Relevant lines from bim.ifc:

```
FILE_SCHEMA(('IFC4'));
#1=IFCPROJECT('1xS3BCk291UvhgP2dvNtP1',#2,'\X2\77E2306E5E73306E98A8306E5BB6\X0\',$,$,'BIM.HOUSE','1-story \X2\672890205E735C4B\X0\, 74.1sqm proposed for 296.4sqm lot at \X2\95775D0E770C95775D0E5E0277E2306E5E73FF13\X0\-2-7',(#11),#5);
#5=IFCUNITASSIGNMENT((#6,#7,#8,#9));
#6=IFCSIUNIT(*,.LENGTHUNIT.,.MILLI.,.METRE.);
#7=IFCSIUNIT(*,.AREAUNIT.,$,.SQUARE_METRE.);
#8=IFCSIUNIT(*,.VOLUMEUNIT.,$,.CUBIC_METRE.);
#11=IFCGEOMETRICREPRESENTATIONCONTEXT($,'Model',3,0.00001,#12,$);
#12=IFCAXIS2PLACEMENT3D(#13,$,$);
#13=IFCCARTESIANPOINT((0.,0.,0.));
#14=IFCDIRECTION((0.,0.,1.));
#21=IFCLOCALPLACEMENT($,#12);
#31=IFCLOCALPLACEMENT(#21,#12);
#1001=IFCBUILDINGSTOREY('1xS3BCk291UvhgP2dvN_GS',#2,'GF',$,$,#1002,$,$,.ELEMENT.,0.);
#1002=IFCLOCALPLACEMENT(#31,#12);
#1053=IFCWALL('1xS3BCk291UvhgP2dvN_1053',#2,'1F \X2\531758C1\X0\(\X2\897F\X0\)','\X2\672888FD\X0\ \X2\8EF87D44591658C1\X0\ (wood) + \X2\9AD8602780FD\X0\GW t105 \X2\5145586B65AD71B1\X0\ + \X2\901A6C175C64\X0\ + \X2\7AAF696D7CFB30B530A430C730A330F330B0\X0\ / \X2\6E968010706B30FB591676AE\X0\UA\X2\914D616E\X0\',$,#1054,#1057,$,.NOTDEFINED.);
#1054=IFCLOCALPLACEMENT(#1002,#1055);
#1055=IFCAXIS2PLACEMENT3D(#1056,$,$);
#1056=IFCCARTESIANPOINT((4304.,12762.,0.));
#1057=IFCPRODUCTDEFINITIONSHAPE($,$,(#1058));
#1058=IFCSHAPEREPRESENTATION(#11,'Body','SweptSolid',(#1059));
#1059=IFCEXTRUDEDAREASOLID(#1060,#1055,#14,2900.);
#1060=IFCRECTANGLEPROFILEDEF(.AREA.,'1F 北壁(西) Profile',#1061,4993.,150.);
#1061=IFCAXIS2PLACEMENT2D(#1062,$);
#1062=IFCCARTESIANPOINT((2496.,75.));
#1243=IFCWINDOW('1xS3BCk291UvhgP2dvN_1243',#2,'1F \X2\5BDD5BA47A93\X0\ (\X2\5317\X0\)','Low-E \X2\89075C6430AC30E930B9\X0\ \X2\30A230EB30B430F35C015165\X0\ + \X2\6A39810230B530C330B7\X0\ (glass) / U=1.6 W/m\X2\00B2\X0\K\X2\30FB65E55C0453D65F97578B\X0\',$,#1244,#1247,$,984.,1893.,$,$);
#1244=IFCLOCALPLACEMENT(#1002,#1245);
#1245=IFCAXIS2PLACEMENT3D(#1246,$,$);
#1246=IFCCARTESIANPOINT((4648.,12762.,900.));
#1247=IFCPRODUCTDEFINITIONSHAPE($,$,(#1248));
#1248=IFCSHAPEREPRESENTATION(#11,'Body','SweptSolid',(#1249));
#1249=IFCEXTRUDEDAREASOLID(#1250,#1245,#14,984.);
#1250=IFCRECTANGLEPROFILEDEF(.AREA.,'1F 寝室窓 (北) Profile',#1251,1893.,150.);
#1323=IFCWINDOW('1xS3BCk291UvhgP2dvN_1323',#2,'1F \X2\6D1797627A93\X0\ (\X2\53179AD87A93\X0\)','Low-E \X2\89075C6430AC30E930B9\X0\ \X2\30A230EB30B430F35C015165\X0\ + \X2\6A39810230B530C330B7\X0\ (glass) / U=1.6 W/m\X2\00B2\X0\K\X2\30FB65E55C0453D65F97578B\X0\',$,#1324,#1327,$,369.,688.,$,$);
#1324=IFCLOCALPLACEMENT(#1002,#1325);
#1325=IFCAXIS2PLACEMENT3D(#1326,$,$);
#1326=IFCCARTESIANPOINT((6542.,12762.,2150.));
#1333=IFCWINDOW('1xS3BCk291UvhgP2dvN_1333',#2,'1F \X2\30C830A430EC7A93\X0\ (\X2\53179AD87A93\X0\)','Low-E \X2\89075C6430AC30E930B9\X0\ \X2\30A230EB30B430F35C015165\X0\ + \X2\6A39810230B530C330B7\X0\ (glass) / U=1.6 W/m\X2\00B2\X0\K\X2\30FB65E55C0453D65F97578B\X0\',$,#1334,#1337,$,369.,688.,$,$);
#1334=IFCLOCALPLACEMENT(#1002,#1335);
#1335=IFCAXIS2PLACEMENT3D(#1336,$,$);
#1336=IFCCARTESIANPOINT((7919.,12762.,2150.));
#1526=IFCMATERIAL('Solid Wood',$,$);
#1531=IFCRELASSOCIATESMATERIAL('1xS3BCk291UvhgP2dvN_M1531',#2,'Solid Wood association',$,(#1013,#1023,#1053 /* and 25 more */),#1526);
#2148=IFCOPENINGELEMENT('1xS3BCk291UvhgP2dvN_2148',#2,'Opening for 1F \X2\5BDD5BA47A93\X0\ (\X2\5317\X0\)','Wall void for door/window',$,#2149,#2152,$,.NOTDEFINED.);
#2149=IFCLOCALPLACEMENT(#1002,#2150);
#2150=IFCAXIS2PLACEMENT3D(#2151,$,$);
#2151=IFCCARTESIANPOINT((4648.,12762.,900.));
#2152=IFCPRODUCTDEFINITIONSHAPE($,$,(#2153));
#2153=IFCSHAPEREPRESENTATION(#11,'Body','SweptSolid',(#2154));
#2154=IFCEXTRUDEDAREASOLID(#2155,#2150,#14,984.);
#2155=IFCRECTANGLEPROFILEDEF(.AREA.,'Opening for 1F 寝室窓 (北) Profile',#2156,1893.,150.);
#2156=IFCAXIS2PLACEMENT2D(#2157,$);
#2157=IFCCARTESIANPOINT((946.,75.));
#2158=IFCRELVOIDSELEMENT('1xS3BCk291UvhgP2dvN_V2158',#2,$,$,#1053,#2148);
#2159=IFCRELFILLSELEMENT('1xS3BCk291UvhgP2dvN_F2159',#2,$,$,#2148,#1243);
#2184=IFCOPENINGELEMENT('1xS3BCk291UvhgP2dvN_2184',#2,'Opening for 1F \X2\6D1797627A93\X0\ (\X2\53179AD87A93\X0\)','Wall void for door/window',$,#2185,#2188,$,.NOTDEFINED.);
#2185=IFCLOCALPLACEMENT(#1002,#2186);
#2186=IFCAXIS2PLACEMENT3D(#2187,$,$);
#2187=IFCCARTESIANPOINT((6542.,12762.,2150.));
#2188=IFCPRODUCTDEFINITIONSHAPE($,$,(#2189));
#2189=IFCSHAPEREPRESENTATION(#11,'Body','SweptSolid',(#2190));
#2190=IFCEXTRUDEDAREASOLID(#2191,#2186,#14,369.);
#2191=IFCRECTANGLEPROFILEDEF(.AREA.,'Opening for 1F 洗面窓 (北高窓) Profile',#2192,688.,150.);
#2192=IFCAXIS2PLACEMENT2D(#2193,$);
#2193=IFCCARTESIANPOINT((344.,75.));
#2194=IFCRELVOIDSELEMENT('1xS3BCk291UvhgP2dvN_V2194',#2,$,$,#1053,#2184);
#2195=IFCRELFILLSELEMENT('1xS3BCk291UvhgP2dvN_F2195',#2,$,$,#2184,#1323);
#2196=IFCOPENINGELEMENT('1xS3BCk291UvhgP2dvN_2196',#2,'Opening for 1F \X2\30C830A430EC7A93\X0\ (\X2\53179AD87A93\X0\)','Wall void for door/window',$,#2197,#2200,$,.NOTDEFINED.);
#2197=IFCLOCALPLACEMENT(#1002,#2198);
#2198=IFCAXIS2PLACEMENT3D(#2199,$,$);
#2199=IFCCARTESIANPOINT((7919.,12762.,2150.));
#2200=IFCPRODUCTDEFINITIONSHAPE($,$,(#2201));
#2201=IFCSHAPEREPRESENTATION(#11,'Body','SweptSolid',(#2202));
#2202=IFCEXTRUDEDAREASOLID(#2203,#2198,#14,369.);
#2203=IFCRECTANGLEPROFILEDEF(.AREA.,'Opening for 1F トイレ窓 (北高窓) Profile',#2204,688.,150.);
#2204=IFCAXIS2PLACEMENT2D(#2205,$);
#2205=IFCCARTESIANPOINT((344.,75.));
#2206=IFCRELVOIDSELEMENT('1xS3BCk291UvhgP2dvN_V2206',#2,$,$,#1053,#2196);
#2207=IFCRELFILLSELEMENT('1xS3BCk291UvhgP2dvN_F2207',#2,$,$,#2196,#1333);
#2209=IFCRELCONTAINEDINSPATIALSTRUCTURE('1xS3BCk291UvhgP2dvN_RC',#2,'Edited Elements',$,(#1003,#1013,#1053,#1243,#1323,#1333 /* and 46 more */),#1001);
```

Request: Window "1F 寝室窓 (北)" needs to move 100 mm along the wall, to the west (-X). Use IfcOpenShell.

```python
import ifcopenshell
import ifcopenshell.api.geometry
import ifcopenshell.util.placement

model = ifcopenshell.open("bim.ifc")

window = model.by_guid("1xS3BCk291UvhgP2dvN_1243")
opening = window.FillsVoids[0].RelatingOpeningElement
wall = opening.VoidsElements[0].RelatingBuildingElement

wall_matrix = ifcopenshell.util.placement.get_local_placement(wall.ObjectPlacement)
shift = wall_matrix[:3, 0] * -100.0
before = ifcopenshell.util.placement.get_local_placement(window.ObjectPlacement)[:3, 3].copy()

# The window is not placed relative to its opening, so move both.
for product in (opening, window):
    matrix = ifcopenshell.util.placement.get_local_placement(product.ObjectPlacement)
    matrix[:3, 3] += shift
    ifcopenshell.api.geometry.edit_object_placement(model, product=product, matrix=matrix, is_si=False)

after = ifcopenshell.util.placement.get_local_placement(window.ObjectPlacement)[:3, 3]
print("window moved by", (after - before).round(3) + 0.0)

model.write("bim_updated.ifc")
```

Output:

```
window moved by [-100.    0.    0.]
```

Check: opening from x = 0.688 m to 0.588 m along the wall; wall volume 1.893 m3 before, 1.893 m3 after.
